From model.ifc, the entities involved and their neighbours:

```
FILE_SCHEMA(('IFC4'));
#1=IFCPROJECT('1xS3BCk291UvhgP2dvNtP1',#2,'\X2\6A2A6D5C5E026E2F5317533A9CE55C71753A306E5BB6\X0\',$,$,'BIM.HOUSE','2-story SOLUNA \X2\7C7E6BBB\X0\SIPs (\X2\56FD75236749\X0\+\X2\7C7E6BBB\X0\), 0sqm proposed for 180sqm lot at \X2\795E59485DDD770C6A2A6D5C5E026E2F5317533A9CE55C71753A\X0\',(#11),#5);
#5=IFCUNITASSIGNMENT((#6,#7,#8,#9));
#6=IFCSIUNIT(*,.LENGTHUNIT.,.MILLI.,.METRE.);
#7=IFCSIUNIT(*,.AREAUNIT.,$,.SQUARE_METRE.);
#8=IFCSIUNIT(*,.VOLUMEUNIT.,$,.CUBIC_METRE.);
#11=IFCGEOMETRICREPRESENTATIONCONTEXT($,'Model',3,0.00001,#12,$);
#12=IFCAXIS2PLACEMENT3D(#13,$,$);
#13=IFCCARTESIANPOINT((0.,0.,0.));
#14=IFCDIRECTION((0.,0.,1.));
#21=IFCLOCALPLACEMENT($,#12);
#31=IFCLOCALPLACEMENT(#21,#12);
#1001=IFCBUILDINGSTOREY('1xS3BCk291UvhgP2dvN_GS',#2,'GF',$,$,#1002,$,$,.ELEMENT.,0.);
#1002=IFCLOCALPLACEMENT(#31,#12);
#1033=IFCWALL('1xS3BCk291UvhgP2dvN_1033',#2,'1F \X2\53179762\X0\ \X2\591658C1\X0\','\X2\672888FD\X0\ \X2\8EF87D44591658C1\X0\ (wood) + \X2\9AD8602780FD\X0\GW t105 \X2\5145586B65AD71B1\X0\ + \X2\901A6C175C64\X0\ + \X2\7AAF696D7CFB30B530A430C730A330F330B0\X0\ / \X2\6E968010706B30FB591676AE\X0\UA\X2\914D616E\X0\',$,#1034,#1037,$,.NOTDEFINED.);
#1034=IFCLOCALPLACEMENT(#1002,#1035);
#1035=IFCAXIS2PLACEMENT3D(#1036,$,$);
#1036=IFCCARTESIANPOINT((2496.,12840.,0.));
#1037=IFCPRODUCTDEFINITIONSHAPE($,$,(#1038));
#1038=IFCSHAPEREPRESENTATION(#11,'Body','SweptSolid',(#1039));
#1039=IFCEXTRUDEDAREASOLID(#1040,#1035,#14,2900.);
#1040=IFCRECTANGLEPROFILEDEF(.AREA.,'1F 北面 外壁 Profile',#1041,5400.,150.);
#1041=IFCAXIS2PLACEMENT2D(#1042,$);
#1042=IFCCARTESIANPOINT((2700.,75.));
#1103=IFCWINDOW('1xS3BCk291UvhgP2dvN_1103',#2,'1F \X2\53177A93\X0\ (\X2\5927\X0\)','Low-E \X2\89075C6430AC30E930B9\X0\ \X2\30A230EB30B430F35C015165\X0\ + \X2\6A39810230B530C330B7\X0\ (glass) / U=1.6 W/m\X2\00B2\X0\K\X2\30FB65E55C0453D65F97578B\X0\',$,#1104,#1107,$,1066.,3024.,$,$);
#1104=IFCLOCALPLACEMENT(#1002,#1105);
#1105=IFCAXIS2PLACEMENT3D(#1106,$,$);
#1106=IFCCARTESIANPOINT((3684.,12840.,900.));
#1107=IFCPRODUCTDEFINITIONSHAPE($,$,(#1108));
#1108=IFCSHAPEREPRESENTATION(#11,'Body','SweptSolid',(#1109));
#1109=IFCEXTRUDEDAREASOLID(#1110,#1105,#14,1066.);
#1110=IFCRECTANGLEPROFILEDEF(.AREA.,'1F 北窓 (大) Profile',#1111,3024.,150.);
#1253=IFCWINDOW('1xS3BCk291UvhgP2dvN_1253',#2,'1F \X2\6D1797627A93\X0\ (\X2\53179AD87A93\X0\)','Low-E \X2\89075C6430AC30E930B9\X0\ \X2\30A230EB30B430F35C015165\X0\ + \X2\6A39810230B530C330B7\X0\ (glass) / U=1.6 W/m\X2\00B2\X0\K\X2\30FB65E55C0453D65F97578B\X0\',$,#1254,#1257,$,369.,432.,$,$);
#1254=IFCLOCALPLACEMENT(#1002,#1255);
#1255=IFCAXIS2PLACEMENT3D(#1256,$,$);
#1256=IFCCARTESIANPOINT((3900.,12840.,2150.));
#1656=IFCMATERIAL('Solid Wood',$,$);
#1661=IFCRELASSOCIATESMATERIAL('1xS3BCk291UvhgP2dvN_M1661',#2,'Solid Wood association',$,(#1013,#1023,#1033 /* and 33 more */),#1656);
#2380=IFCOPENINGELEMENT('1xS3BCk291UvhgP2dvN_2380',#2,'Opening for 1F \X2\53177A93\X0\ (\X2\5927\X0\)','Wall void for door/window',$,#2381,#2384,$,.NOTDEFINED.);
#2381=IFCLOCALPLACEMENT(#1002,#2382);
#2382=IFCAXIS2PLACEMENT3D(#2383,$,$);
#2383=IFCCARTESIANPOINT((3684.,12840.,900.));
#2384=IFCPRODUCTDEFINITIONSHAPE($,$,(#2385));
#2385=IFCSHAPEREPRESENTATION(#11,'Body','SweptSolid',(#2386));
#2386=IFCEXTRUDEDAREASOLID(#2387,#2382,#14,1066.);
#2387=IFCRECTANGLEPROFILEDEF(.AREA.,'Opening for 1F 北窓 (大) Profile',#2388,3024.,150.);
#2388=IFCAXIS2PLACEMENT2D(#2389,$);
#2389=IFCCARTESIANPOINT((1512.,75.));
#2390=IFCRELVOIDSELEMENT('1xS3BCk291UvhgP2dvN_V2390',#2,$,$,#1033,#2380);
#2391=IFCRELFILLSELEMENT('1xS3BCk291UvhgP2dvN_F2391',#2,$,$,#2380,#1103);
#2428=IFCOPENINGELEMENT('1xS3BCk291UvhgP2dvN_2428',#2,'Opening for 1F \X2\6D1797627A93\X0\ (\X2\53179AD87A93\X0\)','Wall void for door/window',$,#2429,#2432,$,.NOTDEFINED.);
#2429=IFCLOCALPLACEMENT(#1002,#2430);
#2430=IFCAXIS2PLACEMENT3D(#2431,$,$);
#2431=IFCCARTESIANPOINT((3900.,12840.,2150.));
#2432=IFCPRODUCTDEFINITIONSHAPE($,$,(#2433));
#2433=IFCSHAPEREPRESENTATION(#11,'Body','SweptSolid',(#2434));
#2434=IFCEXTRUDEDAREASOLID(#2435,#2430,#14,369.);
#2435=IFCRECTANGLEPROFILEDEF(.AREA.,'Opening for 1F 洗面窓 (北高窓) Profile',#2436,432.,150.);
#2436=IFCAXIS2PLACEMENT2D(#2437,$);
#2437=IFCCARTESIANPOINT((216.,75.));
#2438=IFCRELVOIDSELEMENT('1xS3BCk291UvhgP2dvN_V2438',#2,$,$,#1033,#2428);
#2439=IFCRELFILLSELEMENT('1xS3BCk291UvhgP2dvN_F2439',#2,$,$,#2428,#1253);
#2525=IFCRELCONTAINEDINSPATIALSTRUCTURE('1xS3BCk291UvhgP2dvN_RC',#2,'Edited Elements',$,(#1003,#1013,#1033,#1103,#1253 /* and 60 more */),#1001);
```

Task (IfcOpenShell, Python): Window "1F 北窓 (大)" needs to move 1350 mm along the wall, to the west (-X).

```python
import ifcopenshell
import ifcopenshell.api.geometry
import ifcopenshell.util.placement

model = ifcopenshell.open("model.ifc")

window = model.by_guid("1xS3BCk291UvhgP2dvN_1103")
opening = window.FillsVoids[0].RelatingOpeningElement
wall = opening.VoidsElements[0].RelatingBuildingElement

wall_matrix = ifcopenshell.util.placement.get_local_placement(wall.ObjectPlacement)
shift = wall_matrix[:3, 0] * -1350.0
before = ifcopenshell.util.placement.get_local_placement(window.ObjectPlacement)[:3, 3].copy()

# The window is not placed relative to its opening, so move both.
for product in (opening, window):
    matrix = ifcopenshell.util.placement.get_local_placement(product.ObjectPlacement)
    matrix[:3, 3] += shift
    ifcopenshell.api.geometry.edit_object_placement(model, product=product, matrix=matrix, is_si=False)

after = ifcopenshell.util.placement.get_local_placement(window.ObjectPlacement)[:3, 3]
print("window moved by", (after - before).round(3) + 0.0)

model.write("model-out.ifc")
```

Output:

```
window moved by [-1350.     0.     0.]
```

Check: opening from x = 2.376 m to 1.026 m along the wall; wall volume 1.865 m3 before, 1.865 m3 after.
